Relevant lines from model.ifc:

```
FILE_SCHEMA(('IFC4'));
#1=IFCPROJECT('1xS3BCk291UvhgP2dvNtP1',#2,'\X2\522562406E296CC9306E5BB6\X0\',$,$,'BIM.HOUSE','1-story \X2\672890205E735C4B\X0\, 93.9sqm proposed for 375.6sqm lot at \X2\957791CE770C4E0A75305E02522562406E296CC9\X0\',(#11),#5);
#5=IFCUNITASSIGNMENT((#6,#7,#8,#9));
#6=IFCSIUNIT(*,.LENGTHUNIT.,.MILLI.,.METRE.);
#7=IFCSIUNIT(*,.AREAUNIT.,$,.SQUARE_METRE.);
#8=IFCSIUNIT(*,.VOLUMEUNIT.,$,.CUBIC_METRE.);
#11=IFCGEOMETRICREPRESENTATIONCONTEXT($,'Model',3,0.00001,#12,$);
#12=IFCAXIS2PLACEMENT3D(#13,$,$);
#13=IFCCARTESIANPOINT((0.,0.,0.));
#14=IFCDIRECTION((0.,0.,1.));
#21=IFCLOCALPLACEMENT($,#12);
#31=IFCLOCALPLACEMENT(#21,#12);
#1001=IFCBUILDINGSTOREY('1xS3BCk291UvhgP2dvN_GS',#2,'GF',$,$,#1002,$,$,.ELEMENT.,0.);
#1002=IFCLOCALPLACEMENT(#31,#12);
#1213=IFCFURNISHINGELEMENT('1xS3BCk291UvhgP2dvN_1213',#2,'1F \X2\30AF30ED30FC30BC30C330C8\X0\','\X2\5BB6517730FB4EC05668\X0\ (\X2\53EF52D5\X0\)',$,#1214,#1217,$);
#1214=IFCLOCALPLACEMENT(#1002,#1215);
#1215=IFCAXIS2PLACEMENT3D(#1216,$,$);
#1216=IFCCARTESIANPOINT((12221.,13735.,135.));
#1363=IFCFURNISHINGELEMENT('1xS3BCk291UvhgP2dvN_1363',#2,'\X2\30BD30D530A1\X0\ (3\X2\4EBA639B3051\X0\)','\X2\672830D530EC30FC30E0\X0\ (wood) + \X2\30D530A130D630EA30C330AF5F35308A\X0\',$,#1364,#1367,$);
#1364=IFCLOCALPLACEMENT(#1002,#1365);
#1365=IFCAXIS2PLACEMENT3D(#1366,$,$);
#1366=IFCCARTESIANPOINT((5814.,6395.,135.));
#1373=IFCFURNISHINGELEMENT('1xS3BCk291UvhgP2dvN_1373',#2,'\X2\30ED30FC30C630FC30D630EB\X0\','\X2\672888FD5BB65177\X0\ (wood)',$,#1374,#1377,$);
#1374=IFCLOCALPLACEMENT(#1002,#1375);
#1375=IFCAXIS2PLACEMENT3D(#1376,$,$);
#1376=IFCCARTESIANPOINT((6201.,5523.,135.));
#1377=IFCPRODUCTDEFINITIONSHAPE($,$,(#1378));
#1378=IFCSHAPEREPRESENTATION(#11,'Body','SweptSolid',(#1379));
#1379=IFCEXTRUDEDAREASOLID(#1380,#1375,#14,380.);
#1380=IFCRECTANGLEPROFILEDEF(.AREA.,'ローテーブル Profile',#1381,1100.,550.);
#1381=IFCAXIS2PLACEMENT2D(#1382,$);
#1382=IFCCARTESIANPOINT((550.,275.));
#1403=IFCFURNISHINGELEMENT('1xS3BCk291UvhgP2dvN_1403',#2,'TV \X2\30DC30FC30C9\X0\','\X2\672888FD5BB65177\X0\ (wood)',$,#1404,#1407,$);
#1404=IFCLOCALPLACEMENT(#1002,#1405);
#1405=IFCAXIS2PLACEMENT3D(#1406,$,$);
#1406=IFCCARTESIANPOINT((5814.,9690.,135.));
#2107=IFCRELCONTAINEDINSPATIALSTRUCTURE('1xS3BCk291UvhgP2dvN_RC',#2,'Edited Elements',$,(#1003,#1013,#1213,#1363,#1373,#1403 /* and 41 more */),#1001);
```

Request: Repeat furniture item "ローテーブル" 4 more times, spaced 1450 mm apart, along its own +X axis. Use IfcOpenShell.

```python
import ifcopenshell
import ifcopenshell.api.geometry
import ifcopenshell.api.root
import ifcopenshell.util.element
import ifcopenshell.util.placement

model = ifcopenshell.open("model.ifc")


def reuse_history(source, copy):
    """copy_class also copies each property set's owner history, people and application; keep the originals."""
    for rel in copy.IsDefinedBy:
        if rel.is_a("IfcRelDefinesByProperties") and (history := rel.RelatingPropertyDefinition.OwnerHistory):
            rel.RelatingPropertyDefinition.OwnerHistory = source.OwnerHistory
            ifcopenshell.util.element.remove_deep2(model, history)


source = model.by_guid("1xS3BCk291UvhgP2dvN_1373")
base = ifcopenshell.util.placement.get_local_placement(source.ObjectPlacement)
step = base[:3, 0] * 1450.0

for i in range(1, 5):
    copy = ifcopenshell.api.root.copy_class(model, product=source)
    copy.Representation = ifcopenshell.util.element.copy_deep(
        model, source.Representation, exclude=["IfcGeometricRepresentationContext", "IfcRepresentationMap"]
    )
    reuse_history(source, copy)
    matrix = base.copy()
    matrix[:3, 3] += i * step
    print("added at", matrix[:3, 3].round(3) + 0.0)
    ifcopenshell.api.geometry.edit_object_placement(model, product=copy, matrix=matrix, is_si=False)

model.write("model-out.ifc")
```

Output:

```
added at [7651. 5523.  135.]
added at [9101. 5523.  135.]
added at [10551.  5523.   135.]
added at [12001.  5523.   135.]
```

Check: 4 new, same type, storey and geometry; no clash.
